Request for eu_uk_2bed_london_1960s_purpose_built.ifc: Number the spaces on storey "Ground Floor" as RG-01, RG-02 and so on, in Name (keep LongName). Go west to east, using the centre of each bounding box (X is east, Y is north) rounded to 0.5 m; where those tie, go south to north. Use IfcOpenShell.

First a look at what the model holds.

```python
import ifcopenshell
import ifcopenshell.util.element
import ifcopenshell.util.placement

model = ifcopenshell.open("eu_uk_2bed_london_1960s_purpose_built.ifc")
print(model.schema)
storey = next(s for s in model.by_type("IfcBuildingStorey") if s.Name == "Ground Floor")
spaces = [e for e in ifcopenshell.util.element.get_decomposition(storey) if e.is_a("IfcSpace")]
for e in sorted(spaces, key=lambda e: e.id()):
    origin = ifcopenshell.util.placement.get_local_placement(e.ObjectPlacement)[:3, 3]
    print(e.id(), e.Name, e.LongName, origin.round(2) + 0.0, sep=" | ")
```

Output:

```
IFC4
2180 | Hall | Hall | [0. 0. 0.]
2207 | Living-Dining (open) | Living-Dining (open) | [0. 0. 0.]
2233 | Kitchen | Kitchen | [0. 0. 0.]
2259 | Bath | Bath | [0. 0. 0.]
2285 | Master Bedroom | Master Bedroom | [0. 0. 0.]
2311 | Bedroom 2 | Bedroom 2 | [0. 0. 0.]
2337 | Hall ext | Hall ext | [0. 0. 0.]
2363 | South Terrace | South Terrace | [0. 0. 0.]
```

```python
import ifcopenshell
import ifcopenshell.geom
import ifcopenshell.util.element
import ifcopenshell.util.shape

model = ifcopenshell.open("eu_uk_2bed_london_1960s_purpose_built.ifc")
settings = ifcopenshell.geom.settings()
settings.set("use-world-coords", True)


def centre(element):
    shape = ifcopenshell.geom.create_shape(settings, element)
    return ifcopenshell.util.shape.get_bbox_centroid(shape.geometry)


storey = next(s for s in model.by_type("IfcBuildingStorey") if s.Name == "Ground Floor")
spaces = [e for e in ifcopenshell.util.element.get_decomposition(storey) if e.is_a("IfcSpace")]

# Insertion points can sit at a corner or the storey origin, so sort by the geometry (in metres).
centres = {e: centre(e) for e in spaces}
spaces.sort(key=lambda e: (round(centres[e][0] / 0.5), centres[e][1]))

for i, e in enumerate(spaces, start=1):
    number = f"RG-{i:02d}"
    e.Name = number
    print(e.id(), number)

model.write("eu_uk_2bed_london_1960s_purpose_built_edited.ifc")
```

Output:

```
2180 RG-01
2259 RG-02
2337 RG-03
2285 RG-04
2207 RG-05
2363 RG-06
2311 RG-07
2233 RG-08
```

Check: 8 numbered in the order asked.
